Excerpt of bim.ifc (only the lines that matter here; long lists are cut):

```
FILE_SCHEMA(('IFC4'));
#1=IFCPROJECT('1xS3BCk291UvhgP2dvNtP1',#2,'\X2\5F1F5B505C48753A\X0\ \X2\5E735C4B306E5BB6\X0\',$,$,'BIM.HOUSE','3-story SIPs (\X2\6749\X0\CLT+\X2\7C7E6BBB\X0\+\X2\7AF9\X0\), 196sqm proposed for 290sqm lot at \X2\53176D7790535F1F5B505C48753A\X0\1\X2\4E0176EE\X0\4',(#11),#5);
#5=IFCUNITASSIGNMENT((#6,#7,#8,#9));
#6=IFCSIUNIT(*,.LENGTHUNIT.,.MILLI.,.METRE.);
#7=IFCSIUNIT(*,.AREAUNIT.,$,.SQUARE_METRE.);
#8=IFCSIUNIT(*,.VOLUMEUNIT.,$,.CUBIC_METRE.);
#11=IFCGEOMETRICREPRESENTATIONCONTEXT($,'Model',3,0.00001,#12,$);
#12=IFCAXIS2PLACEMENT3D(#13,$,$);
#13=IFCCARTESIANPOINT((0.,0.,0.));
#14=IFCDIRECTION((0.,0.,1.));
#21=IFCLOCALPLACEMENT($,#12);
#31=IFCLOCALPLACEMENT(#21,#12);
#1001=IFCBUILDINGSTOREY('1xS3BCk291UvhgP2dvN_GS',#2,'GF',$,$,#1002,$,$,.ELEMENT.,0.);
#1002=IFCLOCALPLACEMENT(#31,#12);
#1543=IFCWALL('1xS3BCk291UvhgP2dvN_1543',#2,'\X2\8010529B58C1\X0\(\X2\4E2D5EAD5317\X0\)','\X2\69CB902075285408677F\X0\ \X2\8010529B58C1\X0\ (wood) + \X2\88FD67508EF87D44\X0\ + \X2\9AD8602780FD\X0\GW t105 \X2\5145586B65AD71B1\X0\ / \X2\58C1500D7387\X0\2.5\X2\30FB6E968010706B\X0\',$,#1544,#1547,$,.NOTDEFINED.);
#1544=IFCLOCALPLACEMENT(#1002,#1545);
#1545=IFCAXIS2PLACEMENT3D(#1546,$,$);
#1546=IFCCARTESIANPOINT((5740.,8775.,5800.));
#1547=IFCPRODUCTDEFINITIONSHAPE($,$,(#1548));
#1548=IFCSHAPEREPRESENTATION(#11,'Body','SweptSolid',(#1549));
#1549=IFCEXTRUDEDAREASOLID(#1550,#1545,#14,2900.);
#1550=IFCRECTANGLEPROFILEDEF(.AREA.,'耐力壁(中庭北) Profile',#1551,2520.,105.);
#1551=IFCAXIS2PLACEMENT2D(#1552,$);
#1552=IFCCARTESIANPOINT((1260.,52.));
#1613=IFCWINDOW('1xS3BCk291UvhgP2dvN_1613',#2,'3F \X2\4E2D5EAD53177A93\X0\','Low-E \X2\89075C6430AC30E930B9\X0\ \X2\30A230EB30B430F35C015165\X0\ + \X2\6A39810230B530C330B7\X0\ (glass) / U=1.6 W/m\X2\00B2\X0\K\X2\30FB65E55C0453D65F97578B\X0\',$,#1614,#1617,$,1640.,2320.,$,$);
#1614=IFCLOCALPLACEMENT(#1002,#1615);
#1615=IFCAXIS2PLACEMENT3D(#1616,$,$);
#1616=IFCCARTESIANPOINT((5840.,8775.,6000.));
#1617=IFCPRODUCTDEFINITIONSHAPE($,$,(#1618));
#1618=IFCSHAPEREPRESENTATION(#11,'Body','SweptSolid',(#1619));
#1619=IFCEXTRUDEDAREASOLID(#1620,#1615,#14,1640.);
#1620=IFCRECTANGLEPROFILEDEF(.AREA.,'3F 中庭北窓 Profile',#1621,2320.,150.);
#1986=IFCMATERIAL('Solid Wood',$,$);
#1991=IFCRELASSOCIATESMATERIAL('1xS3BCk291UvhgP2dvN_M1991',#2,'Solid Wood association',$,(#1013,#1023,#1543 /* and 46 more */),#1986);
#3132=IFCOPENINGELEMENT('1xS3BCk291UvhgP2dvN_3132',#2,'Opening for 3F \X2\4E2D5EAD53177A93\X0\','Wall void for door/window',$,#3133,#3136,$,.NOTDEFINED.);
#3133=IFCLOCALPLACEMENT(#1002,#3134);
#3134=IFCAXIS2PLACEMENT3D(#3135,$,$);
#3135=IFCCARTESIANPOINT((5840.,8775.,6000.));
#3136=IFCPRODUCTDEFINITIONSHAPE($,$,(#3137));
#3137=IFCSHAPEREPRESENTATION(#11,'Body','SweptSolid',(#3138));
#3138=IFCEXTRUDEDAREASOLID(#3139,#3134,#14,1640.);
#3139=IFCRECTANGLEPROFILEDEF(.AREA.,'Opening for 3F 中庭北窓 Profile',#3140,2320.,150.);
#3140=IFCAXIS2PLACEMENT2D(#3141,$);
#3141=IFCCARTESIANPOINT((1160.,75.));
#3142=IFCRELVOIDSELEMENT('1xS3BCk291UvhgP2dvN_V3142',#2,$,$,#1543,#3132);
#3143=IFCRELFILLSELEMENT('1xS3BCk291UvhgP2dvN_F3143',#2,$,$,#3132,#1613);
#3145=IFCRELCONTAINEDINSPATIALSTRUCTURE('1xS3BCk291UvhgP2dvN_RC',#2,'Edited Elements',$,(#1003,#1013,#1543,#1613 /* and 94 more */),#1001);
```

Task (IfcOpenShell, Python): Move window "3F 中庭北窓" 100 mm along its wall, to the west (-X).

```python
import ifcopenshell
import ifcopenshell.api.geometry
import ifcopenshell.util.placement
import ifcopenshell.util.unit

model = ifcopenshell.open("bim.ifc")
unit_scale = ifcopenshell.util.unit.calculate_unit_scale(model)

window = model.by_guid("1xS3BCk291UvhgP2dvN_1613")
opening = window.FillsVoids[0].RelatingOpeningElement
wall = opening.VoidsElements[0].RelatingBuildingElement

wall_matrix = ifcopenshell.util.placement.get_local_placement(wall.ObjectPlacement)
shift = wall_matrix[:3, 0] * -0.1 / unit_scale
before = ifcopenshell.util.placement.get_local_placement(window.ObjectPlacement)[:3, 3].copy()

# The window is not placed relative to its opening, so move both.
for product in (opening, window):
    matrix = ifcopenshell.util.placement.get_local_placement(product.ObjectPlacement)
    matrix[:3, 3] += shift
    ifcopenshell.api.geometry.edit_object_placement(model, product=product, matrix=matrix, is_si=False)

after = ifcopenshell.util.placement.get_local_placement(window.ObjectPlacement)[:3, 3]
print("window moved by", (after - before).round(3) + 0.0)

model.write("bim_edited.ifc")
```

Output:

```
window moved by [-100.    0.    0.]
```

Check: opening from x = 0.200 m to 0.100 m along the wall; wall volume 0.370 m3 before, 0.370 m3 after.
